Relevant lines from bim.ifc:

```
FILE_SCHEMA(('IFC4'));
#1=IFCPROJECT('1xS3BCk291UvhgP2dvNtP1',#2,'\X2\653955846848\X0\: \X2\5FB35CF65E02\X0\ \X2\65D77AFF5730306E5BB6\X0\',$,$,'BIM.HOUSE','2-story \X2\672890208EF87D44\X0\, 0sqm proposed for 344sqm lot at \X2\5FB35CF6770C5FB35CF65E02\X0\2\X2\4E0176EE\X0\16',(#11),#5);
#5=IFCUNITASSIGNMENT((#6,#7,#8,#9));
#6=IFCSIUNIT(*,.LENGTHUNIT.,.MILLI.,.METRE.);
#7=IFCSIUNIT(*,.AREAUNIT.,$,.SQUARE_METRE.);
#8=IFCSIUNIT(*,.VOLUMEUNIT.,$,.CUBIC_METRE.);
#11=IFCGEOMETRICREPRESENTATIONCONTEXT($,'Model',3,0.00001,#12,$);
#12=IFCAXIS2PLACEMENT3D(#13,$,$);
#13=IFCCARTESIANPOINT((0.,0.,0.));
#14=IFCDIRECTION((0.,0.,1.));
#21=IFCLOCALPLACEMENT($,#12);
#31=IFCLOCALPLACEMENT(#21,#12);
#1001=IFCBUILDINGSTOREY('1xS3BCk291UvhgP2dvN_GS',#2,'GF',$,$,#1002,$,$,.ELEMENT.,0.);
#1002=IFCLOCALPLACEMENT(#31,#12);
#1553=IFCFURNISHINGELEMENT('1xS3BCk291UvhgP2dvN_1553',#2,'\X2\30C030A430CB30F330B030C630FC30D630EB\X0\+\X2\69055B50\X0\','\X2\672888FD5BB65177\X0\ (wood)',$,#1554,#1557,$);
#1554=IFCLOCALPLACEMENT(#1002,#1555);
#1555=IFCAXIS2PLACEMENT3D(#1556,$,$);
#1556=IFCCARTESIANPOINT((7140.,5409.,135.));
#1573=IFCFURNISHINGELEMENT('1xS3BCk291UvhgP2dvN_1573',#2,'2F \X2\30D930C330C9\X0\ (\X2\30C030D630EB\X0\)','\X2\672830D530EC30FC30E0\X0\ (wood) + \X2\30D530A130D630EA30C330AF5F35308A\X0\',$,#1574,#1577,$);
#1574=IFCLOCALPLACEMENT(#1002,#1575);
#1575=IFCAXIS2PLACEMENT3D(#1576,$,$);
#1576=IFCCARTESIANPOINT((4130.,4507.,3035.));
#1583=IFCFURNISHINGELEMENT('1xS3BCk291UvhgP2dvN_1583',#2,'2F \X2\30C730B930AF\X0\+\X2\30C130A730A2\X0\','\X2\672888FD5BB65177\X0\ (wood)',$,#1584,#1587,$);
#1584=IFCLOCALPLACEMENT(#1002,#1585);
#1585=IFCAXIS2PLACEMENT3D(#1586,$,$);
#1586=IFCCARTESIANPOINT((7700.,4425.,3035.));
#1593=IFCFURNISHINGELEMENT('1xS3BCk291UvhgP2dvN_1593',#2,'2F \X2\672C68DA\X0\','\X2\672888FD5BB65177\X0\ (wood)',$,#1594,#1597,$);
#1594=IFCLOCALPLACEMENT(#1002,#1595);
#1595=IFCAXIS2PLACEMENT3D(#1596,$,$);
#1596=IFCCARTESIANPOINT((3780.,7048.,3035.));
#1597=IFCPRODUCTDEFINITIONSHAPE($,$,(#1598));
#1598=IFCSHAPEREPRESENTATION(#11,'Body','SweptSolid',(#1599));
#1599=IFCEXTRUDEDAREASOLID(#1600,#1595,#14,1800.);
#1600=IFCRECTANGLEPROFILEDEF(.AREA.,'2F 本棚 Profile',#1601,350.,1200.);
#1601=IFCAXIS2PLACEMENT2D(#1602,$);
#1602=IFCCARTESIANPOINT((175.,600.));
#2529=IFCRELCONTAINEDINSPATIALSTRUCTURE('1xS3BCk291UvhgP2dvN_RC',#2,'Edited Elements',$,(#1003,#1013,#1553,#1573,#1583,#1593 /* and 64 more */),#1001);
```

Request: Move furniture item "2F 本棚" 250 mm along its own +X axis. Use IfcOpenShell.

```python
import ifcopenshell
import ifcopenshell.api.geometry
import ifcopenshell.util.placement

model = ifcopenshell.open("bim.ifc")

item = model.by_id(1593)
matrix = ifcopenshell.util.placement.get_local_placement(item.ObjectPlacement)
matrix[:3, 3] += matrix[:3, 0] * 250.0
ifcopenshell.api.geometry.edit_object_placement(model, product=item, matrix=matrix, is_si=False)

print(ifcopenshell.util.placement.get_local_placement(item.ObjectPlacement).round(3) + 0.0)

model.write("bim_updated.ifc")
```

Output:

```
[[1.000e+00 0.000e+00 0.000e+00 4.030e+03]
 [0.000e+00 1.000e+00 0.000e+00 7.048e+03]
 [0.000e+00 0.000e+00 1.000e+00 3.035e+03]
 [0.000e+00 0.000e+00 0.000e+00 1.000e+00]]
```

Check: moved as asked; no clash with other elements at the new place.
